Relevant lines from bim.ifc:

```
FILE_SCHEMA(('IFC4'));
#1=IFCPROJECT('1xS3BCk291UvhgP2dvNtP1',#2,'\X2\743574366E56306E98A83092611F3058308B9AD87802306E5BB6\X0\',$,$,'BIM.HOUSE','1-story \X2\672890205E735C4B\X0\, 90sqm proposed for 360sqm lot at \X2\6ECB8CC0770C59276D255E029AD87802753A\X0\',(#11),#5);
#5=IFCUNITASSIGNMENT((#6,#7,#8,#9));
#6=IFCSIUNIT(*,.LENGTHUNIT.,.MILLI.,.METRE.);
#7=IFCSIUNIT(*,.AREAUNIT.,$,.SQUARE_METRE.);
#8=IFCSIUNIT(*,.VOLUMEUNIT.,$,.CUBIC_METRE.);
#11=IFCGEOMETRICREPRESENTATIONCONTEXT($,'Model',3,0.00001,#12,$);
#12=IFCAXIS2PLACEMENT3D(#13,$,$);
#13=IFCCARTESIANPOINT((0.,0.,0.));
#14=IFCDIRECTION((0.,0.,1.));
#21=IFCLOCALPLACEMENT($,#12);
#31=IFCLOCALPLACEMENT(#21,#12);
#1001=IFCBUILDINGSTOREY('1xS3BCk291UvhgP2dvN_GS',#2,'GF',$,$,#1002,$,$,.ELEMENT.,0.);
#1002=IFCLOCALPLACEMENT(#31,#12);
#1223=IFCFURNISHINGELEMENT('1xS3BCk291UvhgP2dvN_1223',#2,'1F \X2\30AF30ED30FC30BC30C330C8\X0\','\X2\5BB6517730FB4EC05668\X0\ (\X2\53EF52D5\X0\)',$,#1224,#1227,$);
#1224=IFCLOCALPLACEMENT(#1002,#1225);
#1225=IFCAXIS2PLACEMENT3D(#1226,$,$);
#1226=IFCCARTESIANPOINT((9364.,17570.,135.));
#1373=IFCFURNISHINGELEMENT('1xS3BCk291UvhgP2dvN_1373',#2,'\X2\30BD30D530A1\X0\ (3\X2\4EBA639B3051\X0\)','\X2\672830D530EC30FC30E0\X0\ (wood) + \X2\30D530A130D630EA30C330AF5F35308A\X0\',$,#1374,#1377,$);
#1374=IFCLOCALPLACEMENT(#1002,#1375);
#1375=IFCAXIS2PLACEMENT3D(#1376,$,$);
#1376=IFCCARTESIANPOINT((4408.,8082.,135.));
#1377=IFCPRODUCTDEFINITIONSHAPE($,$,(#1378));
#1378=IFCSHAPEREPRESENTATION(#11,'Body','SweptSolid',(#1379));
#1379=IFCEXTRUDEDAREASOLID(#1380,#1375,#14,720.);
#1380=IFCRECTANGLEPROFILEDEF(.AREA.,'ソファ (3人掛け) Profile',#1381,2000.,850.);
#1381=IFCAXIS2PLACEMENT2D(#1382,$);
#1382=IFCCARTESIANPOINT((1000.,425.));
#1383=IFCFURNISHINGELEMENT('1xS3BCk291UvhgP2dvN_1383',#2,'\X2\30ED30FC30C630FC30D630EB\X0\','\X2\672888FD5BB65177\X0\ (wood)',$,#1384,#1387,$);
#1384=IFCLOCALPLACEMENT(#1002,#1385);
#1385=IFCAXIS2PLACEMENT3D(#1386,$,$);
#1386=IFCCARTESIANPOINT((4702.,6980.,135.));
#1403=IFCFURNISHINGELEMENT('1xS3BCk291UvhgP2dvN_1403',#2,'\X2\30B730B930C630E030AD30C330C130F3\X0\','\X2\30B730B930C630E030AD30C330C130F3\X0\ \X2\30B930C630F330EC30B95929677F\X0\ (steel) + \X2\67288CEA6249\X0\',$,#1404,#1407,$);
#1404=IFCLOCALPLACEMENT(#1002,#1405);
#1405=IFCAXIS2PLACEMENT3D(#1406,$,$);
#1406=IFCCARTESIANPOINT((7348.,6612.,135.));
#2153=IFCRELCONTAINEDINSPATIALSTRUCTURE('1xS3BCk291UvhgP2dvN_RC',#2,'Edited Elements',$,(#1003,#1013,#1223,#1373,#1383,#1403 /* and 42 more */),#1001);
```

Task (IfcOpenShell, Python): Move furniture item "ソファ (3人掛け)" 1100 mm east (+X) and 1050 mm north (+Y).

```python
import ifcopenshell
import ifcopenshell.api.geometry
import ifcopenshell.util.placement
import ifcopenshell.util.unit

model = ifcopenshell.open("bim.ifc")
unit_scale = ifcopenshell.util.unit.calculate_unit_scale(model)

item = model.by_guid("1xS3BCk291UvhgP2dvN_1373")
matrix = ifcopenshell.util.placement.get_local_placement(item.ObjectPlacement)
matrix[0, 3] += 1.1 / unit_scale
matrix[1, 3] += 1.05 / unit_scale
ifcopenshell.api.geometry.edit_object_placement(model, product=item, matrix=matrix, is_si=False)

print(ifcopenshell.util.placement.get_local_placement(item.ObjectPlacement).round(3) + 0.0)

model.write("bim_rev.ifc")
```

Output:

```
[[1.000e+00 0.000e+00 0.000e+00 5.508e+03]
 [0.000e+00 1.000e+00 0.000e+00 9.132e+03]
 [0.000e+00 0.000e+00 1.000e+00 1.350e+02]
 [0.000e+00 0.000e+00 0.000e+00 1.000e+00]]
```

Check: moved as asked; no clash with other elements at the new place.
